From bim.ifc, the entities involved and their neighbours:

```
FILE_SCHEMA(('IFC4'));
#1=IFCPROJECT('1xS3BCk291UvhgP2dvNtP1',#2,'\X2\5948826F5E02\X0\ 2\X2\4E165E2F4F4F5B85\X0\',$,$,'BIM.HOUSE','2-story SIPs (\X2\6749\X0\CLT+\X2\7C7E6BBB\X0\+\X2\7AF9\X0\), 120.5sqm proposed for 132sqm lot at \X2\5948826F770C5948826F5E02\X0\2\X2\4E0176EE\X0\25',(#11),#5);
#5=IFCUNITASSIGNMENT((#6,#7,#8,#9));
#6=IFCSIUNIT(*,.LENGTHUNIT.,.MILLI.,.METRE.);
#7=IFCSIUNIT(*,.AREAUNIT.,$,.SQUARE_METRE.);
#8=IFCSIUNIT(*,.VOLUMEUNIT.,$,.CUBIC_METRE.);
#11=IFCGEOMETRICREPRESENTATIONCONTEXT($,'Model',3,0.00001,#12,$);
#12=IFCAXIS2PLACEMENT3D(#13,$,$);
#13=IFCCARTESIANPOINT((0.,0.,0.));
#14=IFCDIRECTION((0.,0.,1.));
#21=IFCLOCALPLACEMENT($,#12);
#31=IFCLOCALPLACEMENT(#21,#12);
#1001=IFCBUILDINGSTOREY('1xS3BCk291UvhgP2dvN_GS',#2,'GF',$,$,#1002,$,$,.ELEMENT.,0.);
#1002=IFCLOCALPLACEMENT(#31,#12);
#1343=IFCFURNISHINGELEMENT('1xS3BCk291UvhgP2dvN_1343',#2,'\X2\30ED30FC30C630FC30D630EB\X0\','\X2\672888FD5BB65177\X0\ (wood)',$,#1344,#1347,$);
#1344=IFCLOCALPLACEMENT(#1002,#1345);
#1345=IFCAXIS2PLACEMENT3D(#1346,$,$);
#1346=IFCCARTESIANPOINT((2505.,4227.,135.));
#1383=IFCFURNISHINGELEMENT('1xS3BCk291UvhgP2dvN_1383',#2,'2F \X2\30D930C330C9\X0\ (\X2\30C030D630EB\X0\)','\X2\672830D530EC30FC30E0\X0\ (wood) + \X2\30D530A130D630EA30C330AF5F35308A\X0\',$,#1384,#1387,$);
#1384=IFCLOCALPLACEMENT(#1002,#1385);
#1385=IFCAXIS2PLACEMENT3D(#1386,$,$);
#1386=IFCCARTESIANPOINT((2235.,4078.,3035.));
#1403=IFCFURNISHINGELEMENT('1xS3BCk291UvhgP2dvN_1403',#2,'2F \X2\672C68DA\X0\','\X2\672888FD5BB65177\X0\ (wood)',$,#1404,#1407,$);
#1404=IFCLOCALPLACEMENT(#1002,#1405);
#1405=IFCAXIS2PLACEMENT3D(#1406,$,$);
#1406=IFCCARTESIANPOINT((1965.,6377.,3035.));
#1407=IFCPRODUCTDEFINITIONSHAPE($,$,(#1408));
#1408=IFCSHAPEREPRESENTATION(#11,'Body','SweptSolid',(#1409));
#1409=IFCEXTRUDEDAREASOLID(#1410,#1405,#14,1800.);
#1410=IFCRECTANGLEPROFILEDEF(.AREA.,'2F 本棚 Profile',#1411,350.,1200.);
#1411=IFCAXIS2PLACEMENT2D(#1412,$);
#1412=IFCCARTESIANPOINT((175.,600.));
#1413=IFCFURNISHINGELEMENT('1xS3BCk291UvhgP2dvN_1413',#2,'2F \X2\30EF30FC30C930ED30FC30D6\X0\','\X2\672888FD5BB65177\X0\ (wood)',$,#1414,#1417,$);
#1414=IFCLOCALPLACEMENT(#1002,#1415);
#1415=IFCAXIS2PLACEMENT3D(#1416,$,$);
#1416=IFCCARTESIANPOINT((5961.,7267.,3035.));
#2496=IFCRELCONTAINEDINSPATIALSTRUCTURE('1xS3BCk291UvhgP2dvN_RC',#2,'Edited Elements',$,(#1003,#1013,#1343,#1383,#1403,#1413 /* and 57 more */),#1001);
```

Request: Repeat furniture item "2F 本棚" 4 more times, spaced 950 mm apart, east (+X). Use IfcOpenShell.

```python
import numpy as np
import ifcopenshell
import ifcopenshell.api.geometry
import ifcopenshell.api.root
import ifcopenshell.util.element
import ifcopenshell.util.placement

model = ifcopenshell.open("bim.ifc")


def reuse_history(source, copy):
    """copy_class also copies each property set's owner history, people and application; keep the originals."""
    for rel in copy.IsDefinedBy:
        if rel.is_a("IfcRelDefinesByProperties") and (history := rel.RelatingPropertyDefinition.OwnerHistory):
            rel.RelatingPropertyDefinition.OwnerHistory = source.OwnerHistory
            ifcopenshell.util.element.remove_deep2(model, history)


source = model.by_guid("1xS3BCk291UvhgP2dvN_1403")
base = ifcopenshell.util.placement.get_local_placement(source.ObjectPlacement)
step = np.array([1.0, 0.0, 0.0]) * 950.0

for i in range(1, 5):
    copy = ifcopenshell.api.root.copy_class(model, product=source)
    copy.Representation = ifcopenshell.util.element.copy_deep(
        model, source.Representation, exclude=["IfcGeometricRepresentationContext", "IfcRepresentationMap"]
    )
    reuse_history(source, copy)
    matrix = base.copy()
    matrix[:3, 3] += i * step
    print("added at", matrix[:3, 3].round(3) + 0.0)
    ifcopenshell.api.geometry.edit_object_placement(model, product=copy, matrix=matrix, is_si=False)

model.write("bim_edited.ifc")
```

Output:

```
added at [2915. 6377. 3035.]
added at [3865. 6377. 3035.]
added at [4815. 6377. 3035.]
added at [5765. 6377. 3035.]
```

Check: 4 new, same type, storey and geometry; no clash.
